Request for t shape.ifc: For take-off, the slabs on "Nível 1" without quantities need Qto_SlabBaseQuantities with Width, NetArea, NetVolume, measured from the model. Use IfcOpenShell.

First a look at what the model holds.

```python
import ifcopenshell
import ifcopenshell.util.element
import ifcopenshell.util.unit

model = ifcopenshell.open("t shape.ifc")
print(model.schema)
for unit_type in ("LENGTHUNIT", "AREAUNIT", "VOLUMEUNIT"):
    print(unit_type, ifcopenshell.util.unit.calculate_unit_scale(model, unit_type))
storey = next(s for s in model.by_type("IfcBuildingStorey") if s.Name == "Nível 1")
slabs = [e for e in ifcopenshell.util.element.get_decomposition(storey) if e.is_a("IfcSlab")]
for e in sorted(slabs, key=lambda e: e.id()):
    print(e.id(), e.is_a(), e.Name, list(ifcopenshell.util.element.get_psets(e, qtos_only=True)), sep=" | ")
```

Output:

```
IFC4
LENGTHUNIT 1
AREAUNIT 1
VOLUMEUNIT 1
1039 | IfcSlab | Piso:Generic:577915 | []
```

```python
import ifcopenshell
import ifcopenshell.api.pset
import ifcopenshell.geom
import ifcopenshell.util.element
import ifcopenshell.util.shape
import ifcopenshell.util.unit

model = ifcopenshell.open("t shape.ifc")
unit_scale = ifcopenshell.util.unit.calculate_unit_scale(model)
area_scale = ifcopenshell.util.unit.calculate_unit_scale(model, "AREAUNIT")
volume_scale = ifcopenshell.util.unit.calculate_unit_scale(model, "VOLUMEUNIT")
settings = ifcopenshell.geom.settings()

storey = next(s for s in model.by_type("IfcBuildingStorey") if s.Name == "Nível 1")
slabs = [e for e in ifcopenshell.util.element.get_decomposition(storey) if e.is_a("IfcSlab")]

for e in sorted(slabs, key=lambda e: e.id()):
    if ifcopenshell.util.element.get_psets(e, qtos_only=True, should_inherit=False):
        continue
    # Geometry comes back in metres, in the element's own axes.
    shape = ifcopenshell.geom.create_shape(settings, e)
    values = {
        "Width": ifcopenshell.util.shape.get_z(shape.geometry) / unit_scale,
        "NetArea": ifcopenshell.util.shape.get_footprint_area(shape.geometry) / area_scale,
        "NetVolume": ifcopenshell.util.shape.get_volume(shape.geometry) / volume_scale,
    }
    qto = ifcopenshell.api.pset.add_qto(model, product=e, name="Qto_SlabBaseQuantities")
    ifcopenshell.api.pset.edit_qto(model, qto=qto, properties=values)
    print(e.id(), {k: round(v, 3) for k, v in values.items()})

model.write("t shape_updated.ifc")
```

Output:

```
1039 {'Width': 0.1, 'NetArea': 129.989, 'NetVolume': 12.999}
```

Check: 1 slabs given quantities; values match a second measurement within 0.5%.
